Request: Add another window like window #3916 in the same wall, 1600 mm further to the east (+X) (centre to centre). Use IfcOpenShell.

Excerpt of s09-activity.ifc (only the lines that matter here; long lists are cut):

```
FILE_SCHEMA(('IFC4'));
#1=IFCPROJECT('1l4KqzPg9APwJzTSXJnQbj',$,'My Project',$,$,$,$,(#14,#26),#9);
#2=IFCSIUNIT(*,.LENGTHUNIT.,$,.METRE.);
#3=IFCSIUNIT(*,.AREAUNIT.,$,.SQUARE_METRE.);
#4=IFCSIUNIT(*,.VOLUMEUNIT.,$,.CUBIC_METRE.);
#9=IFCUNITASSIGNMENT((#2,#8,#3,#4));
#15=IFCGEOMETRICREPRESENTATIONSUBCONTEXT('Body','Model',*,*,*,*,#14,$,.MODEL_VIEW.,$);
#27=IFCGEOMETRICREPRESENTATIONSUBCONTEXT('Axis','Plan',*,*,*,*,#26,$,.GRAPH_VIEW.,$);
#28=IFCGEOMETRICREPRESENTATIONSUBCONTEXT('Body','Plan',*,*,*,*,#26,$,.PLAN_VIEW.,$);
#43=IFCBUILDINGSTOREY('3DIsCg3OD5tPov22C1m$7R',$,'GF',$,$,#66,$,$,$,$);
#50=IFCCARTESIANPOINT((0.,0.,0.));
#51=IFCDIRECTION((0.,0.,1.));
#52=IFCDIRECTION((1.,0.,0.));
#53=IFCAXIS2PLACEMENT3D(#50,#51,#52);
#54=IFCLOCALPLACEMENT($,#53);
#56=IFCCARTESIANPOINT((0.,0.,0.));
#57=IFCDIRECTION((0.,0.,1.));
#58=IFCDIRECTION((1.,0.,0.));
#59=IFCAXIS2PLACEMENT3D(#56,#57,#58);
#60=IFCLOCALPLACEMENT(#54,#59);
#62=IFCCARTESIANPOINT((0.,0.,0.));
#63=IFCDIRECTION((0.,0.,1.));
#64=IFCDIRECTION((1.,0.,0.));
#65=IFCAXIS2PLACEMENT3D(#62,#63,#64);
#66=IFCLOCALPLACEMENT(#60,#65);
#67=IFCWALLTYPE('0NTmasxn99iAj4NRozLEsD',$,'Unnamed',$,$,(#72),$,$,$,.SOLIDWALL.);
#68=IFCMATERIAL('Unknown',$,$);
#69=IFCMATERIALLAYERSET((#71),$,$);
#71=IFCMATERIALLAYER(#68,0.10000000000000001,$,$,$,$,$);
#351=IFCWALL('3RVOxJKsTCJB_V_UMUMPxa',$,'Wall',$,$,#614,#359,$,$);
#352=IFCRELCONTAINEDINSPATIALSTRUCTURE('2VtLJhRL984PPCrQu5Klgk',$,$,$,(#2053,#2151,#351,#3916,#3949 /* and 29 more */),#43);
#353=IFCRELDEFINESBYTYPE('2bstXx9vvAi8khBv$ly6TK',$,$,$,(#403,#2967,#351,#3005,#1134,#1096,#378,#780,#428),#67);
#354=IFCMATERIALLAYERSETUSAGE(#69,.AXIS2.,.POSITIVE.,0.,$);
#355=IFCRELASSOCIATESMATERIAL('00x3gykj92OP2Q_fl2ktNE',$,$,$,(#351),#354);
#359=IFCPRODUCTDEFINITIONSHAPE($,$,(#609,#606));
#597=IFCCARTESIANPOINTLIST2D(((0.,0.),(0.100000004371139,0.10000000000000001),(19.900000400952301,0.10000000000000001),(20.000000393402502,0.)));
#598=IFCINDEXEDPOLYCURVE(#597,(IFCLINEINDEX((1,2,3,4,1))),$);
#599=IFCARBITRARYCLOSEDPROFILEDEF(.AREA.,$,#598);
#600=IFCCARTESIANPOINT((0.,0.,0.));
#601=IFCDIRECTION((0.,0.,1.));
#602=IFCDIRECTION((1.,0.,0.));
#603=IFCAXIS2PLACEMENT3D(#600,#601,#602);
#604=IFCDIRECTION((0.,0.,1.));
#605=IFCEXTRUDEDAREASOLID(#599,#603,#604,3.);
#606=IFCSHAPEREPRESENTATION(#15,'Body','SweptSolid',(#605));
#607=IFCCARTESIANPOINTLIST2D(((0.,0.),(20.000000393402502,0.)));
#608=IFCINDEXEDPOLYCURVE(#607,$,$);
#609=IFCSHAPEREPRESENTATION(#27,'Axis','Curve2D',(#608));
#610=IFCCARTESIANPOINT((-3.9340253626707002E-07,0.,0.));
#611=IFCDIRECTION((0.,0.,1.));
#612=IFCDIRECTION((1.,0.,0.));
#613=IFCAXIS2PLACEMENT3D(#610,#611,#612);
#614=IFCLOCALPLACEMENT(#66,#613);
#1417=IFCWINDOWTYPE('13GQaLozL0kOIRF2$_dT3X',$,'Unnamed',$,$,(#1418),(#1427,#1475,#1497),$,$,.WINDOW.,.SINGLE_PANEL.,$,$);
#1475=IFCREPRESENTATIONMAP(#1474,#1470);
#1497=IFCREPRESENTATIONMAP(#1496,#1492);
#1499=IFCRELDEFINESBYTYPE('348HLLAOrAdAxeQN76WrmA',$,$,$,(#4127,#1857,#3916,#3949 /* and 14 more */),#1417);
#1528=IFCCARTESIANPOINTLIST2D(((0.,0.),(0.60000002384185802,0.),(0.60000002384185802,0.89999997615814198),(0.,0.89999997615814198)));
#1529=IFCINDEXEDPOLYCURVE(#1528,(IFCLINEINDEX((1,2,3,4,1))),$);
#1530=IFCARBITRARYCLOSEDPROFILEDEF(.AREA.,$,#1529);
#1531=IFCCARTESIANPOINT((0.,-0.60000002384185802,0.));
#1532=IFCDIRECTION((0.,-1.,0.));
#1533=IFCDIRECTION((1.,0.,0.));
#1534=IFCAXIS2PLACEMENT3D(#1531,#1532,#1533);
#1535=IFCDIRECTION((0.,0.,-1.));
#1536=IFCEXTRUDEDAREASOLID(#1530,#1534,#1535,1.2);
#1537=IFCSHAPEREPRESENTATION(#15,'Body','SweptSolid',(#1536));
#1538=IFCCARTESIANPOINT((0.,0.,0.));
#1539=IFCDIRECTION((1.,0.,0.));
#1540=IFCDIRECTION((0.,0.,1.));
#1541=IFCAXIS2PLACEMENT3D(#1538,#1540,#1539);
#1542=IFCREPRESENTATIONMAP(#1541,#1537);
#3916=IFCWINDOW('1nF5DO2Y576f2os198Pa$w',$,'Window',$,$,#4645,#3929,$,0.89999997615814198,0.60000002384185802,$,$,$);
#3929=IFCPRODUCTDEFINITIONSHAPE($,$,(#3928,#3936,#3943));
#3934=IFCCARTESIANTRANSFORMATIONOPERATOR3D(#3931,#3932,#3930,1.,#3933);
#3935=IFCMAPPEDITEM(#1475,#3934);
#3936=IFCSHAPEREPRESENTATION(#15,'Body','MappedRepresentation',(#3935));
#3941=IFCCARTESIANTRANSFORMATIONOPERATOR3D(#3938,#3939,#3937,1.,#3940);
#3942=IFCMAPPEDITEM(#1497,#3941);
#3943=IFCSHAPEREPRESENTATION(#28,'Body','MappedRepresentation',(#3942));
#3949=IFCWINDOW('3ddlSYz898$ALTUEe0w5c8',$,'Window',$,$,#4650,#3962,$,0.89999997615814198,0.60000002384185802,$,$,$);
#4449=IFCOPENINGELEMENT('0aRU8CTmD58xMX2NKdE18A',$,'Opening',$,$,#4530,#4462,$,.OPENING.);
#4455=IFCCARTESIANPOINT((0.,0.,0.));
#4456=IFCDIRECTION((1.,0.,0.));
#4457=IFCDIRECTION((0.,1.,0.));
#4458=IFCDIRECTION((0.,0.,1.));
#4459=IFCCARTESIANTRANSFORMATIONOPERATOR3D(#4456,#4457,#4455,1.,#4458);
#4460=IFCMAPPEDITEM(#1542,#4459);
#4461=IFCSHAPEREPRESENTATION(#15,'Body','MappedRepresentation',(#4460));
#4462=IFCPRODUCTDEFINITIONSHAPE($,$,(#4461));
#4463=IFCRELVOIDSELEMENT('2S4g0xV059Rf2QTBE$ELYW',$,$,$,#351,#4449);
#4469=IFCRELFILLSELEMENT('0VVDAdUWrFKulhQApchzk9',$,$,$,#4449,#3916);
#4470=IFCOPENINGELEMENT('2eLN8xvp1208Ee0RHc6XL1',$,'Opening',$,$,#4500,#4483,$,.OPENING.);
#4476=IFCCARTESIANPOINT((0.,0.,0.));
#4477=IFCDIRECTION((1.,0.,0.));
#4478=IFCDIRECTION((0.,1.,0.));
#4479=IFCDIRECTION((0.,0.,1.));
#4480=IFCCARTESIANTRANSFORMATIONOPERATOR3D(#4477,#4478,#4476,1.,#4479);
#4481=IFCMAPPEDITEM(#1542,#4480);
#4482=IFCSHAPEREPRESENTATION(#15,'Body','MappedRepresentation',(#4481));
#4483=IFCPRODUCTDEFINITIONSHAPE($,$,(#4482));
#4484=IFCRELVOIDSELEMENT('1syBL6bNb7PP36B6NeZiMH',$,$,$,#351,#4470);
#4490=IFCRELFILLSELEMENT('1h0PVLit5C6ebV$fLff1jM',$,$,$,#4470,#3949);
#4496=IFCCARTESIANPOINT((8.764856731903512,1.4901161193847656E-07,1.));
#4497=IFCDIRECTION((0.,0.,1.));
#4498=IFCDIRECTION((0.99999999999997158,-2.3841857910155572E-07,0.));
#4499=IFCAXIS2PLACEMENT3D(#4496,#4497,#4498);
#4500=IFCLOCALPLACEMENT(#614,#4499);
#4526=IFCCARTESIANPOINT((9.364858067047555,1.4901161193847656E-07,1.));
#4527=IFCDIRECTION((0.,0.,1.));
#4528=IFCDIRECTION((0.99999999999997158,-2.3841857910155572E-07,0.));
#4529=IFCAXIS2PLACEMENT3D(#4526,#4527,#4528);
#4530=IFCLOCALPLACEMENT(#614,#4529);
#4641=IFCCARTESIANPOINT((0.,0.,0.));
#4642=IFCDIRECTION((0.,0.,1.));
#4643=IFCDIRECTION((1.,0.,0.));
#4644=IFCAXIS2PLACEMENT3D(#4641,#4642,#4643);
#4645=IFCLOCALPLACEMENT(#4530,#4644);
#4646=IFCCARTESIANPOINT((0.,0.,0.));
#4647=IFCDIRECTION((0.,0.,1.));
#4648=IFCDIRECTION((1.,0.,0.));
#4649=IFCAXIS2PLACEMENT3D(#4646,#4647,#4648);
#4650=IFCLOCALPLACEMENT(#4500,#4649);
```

```python
import ifcopenshell
import ifcopenshell.api.feature
import ifcopenshell.api.geometry
import ifcopenshell.api.root
import ifcopenshell.geom
import ifcopenshell.util.element
import ifcopenshell.util.placement
import ifcopenshell.util.shape
import ifcopenshell.util.unit

model = ifcopenshell.open("s09-activity.ifc")
unit_scale = ifcopenshell.util.unit.calculate_unit_scale(model)
settings = ifcopenshell.geom.settings()


def volume(element):
    """Net volume in cubic metres, openings subtracted."""
    shape = ifcopenshell.geom.create_shape(settings, element)
    return ifcopenshell.util.shape.get_volume(shape.geometry)


window = model.by_id(3916)
opening = window.FillsVoids[0].RelatingOpeningElement
wall = opening.VoidsElements[0].RelatingBuildingElement
before = volume(wall)
shift = ifcopenshell.util.placement.get_local_placement(wall.ObjectPlacement)[:3, 0] * 1.6 / unit_scale

# copy_class copies the void relationship, type, container and properties, but no geometry.
new_opening = ifcopenshell.api.root.copy_class(model, product=opening)
new_opening.Representation = ifcopenshell.util.element.copy_deep(
    model, opening.Representation, exclude=["IfcGeometricRepresentationContext", "IfcRepresentationMap"]
)
new_window = ifcopenshell.api.root.copy_class(model, product=window)
new_window.Representation = ifcopenshell.util.element.copy_deep(
    model, window.Representation, exclude=["IfcGeometricRepresentationContext", "IfcRepresentationMap"]
)
ifcopenshell.api.feature.add_filling(model, opening=new_opening, element=new_window)

for old, new in ((opening, new_opening), (window, new_window)):
    matrix = ifcopenshell.util.placement.get_local_placement(old.ObjectPlacement)
    matrix[:3, 3] += shift
    ifcopenshell.api.geometry.edit_object_placement(model, product=new, matrix=matrix, is_si=False)

after = volume(wall)

print(f"wall volume {before:.3f} -> {after:.3f} m3")

model.write("s09-activity_rev.ifc")
```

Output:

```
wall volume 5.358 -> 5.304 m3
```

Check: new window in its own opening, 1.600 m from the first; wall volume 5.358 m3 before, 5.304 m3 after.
